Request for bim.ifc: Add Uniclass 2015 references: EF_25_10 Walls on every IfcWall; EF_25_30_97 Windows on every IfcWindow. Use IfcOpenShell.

First a look at what the model holds.

```python
import ifcopenshell

model = ifcopenshell.open("bim.ifc")
print(model.schema)
print("classifications:", [c.Name for c in model.by_type("IfcClassification")])
for ifc_class in ("IfcDoor", "IfcRoof", "IfcStair", "IfcWall", "IfcWindow"):
    print(ifc_class, len(model.by_type(ifc_class)))
```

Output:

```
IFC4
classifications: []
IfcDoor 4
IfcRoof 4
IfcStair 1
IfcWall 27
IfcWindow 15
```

```python
import ifcopenshell
import ifcopenshell.api.classification

model = ifcopenshell.open("bim.ifc")

system = ifcopenshell.api.classification.add_classification(model, classification="Uniclass 2015")

codes = {
    "IfcWall": ("EF_25_10", "Walls"),
    "IfcWindow": ("EF_25_30_97", "Windows"),
}
for ifc_class, (code, name) in codes.items():
    products = model.by_type(ifc_class)
    ifcopenshell.api.classification.add_reference(
        model, products=products, classification=system, identification=code, name=name
    )
    print(code, len(products))

model.write("bim_rev.ifc")
```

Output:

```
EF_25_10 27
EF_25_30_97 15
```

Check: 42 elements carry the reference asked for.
